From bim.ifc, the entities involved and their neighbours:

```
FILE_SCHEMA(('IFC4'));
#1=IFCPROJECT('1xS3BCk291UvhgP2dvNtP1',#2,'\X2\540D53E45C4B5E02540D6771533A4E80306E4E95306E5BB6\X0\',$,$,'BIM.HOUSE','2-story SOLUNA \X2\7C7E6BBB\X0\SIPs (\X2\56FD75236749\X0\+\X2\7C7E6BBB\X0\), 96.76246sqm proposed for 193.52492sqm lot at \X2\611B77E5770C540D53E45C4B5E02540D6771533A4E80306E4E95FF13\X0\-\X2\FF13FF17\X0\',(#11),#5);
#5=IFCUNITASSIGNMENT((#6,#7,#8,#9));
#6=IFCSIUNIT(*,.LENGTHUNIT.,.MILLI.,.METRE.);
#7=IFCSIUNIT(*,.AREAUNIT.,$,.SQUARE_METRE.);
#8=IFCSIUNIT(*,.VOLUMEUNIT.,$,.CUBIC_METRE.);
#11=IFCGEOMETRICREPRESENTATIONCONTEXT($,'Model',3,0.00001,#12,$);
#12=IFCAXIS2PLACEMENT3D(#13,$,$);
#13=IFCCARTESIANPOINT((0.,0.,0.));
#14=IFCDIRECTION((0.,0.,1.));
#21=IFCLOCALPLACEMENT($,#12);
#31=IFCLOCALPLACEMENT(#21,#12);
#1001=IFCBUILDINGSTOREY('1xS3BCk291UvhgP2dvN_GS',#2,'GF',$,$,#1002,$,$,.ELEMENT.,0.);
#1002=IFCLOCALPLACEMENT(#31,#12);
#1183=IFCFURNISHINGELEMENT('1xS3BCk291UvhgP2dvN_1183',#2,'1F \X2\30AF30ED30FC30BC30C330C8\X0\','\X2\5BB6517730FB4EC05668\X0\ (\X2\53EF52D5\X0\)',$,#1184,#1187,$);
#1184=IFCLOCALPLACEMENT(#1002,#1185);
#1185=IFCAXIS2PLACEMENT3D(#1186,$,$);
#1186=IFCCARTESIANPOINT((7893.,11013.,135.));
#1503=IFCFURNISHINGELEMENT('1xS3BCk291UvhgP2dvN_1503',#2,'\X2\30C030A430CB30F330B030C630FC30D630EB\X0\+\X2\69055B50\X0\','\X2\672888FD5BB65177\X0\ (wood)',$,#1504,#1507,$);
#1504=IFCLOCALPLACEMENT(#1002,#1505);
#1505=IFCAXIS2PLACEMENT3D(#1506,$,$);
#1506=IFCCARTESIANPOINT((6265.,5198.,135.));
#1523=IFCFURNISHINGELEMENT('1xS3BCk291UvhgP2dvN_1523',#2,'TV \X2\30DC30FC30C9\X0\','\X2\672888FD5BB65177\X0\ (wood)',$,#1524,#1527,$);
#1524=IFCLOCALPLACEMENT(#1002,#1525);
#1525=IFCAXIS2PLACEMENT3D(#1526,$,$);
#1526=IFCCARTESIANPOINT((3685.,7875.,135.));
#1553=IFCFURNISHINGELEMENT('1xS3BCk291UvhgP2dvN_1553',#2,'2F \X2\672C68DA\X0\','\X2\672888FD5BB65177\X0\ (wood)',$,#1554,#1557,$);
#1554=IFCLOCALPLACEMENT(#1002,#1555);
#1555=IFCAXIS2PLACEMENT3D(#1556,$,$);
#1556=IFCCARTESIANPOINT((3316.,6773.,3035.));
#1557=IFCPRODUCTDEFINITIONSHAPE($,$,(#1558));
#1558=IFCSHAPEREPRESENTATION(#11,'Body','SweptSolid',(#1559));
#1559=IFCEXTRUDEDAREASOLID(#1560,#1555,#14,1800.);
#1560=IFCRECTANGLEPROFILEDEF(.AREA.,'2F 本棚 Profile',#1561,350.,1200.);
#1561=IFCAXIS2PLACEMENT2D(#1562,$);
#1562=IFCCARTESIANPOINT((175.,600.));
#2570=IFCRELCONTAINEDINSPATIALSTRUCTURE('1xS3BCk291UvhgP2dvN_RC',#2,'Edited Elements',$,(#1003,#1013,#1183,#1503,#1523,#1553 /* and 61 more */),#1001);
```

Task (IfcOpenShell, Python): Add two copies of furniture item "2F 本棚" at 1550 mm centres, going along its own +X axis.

```python
import ifcopenshell
import ifcopenshell.api.geometry
import ifcopenshell.api.root
import ifcopenshell.util.element
import ifcopenshell.util.placement

model = ifcopenshell.open("bim.ifc")


def reuse_history(source, copy):
    """copy_class also copies each property set's owner history, people and application; keep the originals."""
    for rel in copy.IsDefinedBy:
        if rel.is_a("IfcRelDefinesByProperties") and (history := rel.RelatingPropertyDefinition.OwnerHistory):
            rel.RelatingPropertyDefinition.OwnerHistory = source.OwnerHistory
            ifcopenshell.util.element.remove_deep2(model, history)


source = model.by_guid("1xS3BCk291UvhgP2dvN_1553")
base = ifcopenshell.util.placement.get_local_placement(source.ObjectPlacement)
step = base[:3, 0] * 1550.0

for i in range(1, 3):
    copy = ifcopenshell.api.root.copy_class(model, product=source)
    copy.Representation = ifcopenshell.util.element.copy_deep(
        model, source.Representation, exclude=["IfcGeometricRepresentationContext", "IfcRepresentationMap"]
    )
    reuse_history(source, copy)
    matrix = base.copy()
    matrix[:3, 3] += i * step
    print("added at", matrix[:3, 3].round(3) + 0.0)
    ifcopenshell.api.geometry.edit_object_placement(model, product=copy, matrix=matrix, is_si=False)

model.write("bim-out.ifc")
```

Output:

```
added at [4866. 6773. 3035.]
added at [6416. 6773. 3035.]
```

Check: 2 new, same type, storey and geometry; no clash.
